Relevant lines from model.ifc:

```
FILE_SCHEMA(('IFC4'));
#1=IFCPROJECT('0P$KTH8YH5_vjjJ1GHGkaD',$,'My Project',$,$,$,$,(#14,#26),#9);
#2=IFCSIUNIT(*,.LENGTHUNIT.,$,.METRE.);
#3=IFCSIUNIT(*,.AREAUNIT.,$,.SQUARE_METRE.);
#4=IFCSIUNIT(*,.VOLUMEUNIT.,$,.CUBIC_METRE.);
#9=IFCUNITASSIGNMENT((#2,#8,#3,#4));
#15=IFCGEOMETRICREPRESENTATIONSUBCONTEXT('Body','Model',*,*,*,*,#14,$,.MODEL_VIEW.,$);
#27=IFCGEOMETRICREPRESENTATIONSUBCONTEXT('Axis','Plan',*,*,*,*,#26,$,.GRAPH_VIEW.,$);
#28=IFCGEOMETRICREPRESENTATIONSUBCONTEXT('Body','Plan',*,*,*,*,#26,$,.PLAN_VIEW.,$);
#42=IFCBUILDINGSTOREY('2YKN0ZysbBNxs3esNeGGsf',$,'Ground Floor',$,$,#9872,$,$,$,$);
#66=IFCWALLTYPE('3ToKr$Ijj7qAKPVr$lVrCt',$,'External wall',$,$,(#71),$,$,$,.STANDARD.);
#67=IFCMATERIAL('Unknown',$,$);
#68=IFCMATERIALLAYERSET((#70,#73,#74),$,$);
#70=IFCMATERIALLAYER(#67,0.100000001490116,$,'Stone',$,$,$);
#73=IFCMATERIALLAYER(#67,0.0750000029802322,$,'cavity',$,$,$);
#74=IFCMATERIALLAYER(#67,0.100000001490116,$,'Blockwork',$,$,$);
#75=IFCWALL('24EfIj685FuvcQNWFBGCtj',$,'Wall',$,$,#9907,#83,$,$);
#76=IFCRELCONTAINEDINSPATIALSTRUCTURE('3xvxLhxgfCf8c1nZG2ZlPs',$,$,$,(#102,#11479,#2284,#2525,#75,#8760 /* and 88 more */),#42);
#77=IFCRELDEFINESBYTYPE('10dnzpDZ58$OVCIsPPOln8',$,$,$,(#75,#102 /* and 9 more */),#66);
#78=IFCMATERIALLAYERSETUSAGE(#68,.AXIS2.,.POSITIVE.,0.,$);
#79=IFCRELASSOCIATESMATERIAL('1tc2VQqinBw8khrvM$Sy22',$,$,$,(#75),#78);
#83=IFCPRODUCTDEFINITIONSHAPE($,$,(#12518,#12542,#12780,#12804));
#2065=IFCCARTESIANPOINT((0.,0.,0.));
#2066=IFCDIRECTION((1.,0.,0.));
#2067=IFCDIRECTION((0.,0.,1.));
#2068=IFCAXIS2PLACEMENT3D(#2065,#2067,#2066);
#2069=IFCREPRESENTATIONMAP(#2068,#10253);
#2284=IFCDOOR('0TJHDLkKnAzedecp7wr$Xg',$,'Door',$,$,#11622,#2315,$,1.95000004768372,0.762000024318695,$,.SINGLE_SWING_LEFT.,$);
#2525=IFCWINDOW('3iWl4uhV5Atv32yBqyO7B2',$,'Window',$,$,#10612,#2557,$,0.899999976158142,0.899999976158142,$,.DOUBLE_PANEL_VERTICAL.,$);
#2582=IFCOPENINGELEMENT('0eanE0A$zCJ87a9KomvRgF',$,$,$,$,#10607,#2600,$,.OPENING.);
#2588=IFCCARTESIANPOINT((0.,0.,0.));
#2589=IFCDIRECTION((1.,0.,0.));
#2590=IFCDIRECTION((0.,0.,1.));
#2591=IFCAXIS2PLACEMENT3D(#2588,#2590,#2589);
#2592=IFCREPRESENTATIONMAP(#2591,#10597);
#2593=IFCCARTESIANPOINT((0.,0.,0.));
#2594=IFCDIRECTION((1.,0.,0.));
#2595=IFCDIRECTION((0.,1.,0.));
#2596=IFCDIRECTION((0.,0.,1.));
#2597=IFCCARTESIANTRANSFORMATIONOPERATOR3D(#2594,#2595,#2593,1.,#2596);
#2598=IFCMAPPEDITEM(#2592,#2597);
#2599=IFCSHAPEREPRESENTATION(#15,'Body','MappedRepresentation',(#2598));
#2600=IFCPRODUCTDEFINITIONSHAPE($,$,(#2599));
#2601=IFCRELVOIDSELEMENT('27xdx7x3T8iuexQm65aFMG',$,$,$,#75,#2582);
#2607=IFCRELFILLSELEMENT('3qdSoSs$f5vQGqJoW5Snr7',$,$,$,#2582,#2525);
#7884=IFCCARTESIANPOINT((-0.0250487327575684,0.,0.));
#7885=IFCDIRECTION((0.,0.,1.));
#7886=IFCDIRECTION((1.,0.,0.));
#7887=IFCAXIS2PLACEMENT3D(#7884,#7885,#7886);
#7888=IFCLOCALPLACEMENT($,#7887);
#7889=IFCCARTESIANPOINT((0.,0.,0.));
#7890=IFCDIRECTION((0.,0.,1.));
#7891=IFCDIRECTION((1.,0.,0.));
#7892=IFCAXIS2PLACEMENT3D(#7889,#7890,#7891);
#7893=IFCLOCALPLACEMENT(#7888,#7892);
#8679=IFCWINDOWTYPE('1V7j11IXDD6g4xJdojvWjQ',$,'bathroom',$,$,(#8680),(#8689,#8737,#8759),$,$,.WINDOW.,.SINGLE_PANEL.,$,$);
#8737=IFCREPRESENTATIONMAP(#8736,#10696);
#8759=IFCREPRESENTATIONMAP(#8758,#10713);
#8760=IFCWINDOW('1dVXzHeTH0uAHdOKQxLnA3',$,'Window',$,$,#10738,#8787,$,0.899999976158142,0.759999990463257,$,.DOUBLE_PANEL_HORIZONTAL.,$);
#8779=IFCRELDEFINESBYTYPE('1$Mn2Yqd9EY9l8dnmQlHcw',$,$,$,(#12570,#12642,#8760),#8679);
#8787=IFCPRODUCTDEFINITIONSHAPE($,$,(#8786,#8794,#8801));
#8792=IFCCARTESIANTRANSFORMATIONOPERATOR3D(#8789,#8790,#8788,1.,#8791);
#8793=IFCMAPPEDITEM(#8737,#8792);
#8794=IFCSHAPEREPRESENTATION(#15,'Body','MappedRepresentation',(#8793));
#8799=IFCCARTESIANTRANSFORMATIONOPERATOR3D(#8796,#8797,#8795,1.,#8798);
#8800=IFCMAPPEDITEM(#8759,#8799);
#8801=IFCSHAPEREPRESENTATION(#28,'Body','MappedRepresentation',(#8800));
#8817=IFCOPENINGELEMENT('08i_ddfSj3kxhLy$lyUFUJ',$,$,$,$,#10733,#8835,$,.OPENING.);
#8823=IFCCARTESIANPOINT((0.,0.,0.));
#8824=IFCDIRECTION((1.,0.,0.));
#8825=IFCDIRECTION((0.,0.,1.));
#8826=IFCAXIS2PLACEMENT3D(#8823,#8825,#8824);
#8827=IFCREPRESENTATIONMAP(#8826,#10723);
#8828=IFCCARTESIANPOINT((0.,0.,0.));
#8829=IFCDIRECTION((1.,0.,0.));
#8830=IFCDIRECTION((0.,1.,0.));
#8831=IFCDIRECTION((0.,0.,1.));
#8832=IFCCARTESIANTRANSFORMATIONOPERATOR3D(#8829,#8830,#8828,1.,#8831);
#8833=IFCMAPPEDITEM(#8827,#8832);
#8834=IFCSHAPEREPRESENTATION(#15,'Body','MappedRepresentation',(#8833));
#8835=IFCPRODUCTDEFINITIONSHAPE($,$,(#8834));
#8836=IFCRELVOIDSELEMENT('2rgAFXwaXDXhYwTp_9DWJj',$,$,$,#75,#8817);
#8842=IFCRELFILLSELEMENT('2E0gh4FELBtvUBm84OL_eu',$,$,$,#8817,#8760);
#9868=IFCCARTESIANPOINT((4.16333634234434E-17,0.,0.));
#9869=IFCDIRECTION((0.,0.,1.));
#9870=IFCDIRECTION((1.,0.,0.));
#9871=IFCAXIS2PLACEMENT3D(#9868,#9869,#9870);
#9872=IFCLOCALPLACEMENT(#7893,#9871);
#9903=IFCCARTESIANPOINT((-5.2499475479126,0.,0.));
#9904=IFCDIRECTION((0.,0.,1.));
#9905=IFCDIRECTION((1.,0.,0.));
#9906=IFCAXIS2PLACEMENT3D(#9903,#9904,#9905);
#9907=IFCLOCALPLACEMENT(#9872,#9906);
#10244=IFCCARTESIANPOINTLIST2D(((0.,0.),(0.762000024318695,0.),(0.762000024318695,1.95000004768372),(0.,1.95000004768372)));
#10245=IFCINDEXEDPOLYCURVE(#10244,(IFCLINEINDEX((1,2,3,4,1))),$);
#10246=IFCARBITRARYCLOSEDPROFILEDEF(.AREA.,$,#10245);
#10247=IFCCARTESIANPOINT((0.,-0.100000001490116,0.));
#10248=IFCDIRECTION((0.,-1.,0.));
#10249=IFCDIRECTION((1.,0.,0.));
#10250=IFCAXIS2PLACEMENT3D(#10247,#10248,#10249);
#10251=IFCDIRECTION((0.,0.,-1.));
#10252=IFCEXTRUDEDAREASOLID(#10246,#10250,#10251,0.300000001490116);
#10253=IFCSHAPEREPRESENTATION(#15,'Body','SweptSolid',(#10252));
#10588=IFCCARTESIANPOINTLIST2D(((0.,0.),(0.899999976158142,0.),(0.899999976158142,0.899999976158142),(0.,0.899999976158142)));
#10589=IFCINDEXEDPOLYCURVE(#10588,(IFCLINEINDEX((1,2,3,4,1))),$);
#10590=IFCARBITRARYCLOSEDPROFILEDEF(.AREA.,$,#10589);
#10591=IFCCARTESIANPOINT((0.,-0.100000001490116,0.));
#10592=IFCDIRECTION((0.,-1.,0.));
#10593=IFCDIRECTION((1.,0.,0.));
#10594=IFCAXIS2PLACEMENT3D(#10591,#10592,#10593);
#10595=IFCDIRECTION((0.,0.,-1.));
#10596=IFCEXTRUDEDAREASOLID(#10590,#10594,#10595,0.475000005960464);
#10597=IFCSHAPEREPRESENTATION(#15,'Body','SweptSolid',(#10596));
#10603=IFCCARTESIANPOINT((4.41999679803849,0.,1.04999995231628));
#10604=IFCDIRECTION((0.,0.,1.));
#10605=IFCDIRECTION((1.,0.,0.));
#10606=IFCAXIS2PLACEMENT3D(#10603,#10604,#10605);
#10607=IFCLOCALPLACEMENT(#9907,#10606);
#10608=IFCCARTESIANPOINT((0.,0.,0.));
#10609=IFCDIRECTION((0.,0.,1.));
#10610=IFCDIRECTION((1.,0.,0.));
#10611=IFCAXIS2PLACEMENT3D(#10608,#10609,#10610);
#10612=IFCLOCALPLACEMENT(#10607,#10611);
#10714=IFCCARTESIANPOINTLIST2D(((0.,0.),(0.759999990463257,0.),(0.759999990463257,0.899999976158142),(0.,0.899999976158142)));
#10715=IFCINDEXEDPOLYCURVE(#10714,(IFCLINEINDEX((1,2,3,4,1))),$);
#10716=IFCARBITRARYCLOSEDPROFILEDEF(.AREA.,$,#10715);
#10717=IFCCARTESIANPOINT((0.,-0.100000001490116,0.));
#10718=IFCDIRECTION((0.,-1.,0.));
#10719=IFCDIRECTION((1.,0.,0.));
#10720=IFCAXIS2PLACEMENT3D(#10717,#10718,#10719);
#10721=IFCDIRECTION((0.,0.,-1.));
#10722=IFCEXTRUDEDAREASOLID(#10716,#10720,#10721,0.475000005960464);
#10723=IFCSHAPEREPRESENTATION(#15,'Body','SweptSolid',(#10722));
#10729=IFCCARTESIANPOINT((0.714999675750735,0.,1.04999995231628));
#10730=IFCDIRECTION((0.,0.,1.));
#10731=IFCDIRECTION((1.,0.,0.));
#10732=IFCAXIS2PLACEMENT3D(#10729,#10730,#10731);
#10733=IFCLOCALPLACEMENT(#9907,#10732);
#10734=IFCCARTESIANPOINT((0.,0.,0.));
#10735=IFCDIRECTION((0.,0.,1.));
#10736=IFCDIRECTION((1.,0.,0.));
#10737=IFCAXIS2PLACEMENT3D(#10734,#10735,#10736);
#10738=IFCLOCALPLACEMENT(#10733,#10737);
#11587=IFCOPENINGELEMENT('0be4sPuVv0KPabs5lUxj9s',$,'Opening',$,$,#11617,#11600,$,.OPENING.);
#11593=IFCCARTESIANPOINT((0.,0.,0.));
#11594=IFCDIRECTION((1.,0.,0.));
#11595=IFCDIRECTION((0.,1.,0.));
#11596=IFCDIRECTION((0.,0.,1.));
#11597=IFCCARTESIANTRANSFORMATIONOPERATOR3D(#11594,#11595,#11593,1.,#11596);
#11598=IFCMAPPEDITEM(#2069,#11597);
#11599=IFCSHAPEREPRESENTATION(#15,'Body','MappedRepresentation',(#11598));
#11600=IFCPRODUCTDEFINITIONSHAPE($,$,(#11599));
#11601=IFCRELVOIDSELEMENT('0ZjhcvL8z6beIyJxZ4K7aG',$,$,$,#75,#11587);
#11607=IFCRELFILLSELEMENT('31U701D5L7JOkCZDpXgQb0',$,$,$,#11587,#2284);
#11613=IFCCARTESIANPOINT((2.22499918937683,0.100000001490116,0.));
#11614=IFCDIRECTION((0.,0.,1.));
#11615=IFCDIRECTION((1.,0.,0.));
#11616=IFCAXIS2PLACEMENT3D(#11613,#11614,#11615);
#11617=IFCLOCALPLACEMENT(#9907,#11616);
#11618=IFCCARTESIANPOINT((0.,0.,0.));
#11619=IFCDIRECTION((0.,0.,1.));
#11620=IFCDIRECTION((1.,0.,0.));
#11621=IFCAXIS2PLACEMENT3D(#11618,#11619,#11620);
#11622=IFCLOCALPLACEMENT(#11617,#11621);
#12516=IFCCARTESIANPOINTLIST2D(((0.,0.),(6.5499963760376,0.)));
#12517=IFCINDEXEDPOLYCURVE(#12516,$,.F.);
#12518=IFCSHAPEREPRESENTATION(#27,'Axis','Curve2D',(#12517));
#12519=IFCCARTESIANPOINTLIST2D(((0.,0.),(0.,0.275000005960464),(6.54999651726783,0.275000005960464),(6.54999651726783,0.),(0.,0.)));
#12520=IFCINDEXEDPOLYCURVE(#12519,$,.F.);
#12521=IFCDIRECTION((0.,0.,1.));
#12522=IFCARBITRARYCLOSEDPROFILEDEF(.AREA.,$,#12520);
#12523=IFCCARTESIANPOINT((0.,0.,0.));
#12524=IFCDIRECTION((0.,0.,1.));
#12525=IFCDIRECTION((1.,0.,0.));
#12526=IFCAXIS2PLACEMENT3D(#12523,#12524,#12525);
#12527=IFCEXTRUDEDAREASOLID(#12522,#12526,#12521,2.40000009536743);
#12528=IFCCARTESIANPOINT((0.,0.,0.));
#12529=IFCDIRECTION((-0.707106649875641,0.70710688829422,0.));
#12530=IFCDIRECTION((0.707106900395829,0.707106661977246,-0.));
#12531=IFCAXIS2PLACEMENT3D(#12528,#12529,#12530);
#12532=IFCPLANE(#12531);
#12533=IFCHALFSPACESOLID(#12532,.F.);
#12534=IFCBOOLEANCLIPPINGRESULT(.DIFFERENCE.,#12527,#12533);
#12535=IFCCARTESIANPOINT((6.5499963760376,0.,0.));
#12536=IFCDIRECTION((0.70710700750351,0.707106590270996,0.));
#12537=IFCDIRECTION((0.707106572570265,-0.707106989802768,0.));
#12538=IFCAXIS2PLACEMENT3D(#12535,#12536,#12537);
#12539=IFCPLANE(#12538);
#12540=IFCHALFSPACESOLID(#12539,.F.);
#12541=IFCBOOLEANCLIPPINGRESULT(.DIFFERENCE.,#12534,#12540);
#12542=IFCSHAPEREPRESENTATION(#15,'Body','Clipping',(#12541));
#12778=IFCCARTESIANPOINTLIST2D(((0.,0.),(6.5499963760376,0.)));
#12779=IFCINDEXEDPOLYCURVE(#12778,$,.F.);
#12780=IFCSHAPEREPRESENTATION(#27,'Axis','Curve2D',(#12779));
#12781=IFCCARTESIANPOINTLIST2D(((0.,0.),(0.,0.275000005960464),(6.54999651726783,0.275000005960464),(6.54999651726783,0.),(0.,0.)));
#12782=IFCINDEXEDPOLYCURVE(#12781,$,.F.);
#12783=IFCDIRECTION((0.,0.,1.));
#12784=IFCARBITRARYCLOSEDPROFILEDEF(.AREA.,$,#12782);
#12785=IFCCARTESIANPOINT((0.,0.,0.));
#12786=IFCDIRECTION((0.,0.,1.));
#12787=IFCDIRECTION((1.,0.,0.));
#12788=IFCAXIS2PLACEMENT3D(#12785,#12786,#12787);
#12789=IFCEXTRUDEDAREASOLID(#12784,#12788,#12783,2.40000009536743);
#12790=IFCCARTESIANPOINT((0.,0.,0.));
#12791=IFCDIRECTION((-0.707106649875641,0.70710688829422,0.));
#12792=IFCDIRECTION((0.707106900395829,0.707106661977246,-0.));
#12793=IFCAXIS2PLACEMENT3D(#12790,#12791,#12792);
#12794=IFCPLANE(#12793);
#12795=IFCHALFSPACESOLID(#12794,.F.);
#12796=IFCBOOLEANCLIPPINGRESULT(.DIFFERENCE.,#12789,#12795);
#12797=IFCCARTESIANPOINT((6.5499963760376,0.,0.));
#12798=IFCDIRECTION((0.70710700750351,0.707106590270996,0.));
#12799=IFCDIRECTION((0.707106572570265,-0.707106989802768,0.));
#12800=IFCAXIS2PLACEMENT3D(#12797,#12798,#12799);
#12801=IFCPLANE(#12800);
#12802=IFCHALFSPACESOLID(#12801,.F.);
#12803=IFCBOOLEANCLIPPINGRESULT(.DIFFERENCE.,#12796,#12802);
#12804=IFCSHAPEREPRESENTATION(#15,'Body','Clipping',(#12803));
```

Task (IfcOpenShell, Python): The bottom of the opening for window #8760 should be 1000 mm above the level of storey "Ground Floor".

```python
import numpy as np
import ifcopenshell
import ifcopenshell.api.geometry
import ifcopenshell.geom
import ifcopenshell.util.element
import ifcopenshell.util.placement
import ifcopenshell.util.shape
import ifcopenshell.util.unit

model = ifcopenshell.open("model.ifc")
unit_scale = ifcopenshell.util.unit.calculate_unit_scale(model)

window = model.by_id(8760)
opening = window.FillsVoids[0].RelatingOpeningElement
storey = ifcopenshell.util.element.get_container(window, ifc_class="IfcBuildingStorey")
level = ifcopenshell.util.placement.get_local_placement(storey.ObjectPlacement)[2, 3]

# The opening's origin need not be at the sill, so measure its lowest point.
shape = ifcopenshell.geom.create_shape(ifcopenshell.geom.settings(), opening)
bottom = ifcopenshell.util.shape.get_shape_bottom_elevation(shape, shape.geometry) / unit_scale
dz = level + 1.0 - bottom

shift = np.array([0.0, 0.0, dz])
# The window is placed relative to its opening, so it follows when the opening moves.
matrix = ifcopenshell.util.placement.get_local_placement(opening.ObjectPlacement)
matrix[:3, 3] += shift
ifcopenshell.api.geometry.edit_object_placement(
    model, product=opening, matrix=matrix, is_si=False, should_transform_children=True
)

print(f"moved by {dz * unit_scale:+.3f} m")

model.write("model_rev.ifc")
```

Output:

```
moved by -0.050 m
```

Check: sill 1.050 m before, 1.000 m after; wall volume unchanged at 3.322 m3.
